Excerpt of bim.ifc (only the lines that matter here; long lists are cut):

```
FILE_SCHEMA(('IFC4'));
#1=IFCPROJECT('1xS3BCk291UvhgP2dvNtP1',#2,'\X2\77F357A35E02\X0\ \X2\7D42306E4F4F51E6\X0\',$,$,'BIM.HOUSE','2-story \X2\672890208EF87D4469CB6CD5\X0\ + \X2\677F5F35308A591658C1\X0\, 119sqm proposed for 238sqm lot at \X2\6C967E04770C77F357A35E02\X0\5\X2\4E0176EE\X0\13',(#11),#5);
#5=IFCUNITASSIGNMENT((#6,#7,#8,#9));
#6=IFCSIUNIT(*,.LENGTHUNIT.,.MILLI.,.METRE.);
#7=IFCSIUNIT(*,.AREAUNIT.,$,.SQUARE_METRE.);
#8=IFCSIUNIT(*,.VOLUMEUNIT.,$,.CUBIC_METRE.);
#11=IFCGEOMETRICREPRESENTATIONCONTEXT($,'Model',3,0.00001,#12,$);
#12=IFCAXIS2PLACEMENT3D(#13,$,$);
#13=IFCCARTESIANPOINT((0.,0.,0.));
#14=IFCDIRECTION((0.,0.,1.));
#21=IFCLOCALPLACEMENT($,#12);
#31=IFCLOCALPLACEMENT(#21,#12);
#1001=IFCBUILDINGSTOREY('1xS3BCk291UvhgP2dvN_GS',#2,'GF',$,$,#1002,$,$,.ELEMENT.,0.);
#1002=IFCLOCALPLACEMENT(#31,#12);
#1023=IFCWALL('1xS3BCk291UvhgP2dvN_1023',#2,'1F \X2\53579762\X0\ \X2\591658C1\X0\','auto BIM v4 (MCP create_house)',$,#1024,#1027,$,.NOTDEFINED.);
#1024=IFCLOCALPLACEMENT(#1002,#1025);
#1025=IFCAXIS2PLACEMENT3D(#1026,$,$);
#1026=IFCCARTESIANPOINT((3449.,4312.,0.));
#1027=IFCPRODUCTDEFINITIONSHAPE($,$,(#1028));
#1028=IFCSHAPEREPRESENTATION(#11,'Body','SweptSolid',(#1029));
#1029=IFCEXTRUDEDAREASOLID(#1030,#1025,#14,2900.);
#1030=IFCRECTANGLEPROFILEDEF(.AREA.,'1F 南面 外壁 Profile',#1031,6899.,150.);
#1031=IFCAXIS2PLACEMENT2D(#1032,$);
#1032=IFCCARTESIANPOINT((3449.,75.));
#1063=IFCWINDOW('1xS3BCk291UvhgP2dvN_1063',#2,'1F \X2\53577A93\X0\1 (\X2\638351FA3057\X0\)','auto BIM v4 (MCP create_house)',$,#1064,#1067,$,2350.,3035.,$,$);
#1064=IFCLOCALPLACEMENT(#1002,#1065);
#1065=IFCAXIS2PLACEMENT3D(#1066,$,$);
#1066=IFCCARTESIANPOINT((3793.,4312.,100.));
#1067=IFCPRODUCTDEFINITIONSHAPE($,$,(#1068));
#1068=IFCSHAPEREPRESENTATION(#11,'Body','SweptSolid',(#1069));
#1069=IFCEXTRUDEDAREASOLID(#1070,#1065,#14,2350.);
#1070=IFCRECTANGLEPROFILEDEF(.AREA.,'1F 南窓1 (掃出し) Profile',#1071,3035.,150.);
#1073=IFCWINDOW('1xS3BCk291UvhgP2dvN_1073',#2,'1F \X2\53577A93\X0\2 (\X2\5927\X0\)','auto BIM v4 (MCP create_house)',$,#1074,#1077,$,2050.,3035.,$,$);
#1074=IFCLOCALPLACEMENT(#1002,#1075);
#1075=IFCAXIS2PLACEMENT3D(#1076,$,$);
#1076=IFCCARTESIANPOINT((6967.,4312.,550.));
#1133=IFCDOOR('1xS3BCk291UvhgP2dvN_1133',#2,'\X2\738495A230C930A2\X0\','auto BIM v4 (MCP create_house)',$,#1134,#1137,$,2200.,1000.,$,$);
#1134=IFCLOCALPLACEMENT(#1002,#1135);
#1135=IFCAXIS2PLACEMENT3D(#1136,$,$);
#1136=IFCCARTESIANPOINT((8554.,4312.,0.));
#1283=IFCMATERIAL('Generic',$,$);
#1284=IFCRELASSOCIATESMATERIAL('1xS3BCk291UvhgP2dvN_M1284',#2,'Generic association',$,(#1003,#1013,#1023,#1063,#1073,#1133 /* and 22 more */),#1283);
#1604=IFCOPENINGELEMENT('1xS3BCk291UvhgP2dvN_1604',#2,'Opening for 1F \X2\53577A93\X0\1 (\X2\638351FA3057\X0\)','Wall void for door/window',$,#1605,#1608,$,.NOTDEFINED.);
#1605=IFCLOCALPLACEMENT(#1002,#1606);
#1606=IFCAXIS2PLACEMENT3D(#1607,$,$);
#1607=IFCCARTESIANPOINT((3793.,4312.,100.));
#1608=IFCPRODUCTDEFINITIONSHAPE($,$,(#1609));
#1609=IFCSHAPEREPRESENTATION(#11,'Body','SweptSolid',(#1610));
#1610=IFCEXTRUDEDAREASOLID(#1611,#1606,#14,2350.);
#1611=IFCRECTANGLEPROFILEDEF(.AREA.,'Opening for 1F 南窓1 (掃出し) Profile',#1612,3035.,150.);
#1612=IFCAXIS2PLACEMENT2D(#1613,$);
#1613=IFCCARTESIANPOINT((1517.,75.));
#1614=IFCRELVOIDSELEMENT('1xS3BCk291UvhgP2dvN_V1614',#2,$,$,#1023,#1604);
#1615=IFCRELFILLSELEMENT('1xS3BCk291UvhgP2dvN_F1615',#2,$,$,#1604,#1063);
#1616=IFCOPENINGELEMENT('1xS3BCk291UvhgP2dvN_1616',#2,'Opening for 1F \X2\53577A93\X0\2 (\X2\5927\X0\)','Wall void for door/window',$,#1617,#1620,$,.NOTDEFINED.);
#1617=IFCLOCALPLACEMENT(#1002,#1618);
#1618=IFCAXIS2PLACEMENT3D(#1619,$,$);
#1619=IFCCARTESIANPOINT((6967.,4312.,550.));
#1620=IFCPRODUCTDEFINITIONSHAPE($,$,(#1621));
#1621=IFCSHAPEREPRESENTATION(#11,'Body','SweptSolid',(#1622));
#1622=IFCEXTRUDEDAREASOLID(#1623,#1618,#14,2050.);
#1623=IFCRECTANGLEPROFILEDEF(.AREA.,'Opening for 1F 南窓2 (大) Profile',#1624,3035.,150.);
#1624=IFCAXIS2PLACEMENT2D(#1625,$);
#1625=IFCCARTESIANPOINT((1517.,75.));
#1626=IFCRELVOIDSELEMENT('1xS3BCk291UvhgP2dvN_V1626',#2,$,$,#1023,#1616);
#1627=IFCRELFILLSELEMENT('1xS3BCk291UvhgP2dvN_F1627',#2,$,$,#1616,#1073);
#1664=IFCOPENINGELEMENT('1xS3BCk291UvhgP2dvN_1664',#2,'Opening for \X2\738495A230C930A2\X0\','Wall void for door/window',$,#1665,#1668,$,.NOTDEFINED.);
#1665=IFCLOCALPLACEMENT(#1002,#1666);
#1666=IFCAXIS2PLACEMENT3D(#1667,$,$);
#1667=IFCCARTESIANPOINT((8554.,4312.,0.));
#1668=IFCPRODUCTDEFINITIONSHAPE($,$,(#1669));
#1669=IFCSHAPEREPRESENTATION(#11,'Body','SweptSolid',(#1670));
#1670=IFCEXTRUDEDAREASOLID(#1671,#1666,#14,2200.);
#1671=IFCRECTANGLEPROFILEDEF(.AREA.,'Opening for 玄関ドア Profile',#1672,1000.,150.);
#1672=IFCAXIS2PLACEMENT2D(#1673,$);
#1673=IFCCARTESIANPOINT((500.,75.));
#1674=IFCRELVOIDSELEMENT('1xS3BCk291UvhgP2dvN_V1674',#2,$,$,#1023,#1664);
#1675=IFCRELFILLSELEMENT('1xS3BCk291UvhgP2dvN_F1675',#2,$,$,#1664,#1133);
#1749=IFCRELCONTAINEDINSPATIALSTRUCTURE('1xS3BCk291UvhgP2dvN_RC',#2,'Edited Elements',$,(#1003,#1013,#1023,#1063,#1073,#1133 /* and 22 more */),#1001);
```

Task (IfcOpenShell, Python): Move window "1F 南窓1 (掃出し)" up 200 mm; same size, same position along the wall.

```python
import numpy as np
import ifcopenshell
import ifcopenshell.api.geometry
import ifcopenshell.util.placement
import ifcopenshell.util.unit

model = ifcopenshell.open("bim.ifc")
unit_scale = ifcopenshell.util.unit.calculate_unit_scale(model)

window = model.by_id(1063)
opening = window.FillsVoids[0].RelatingOpeningElement
dz = 200.0

shift = np.array([0.0, 0.0, dz])
# The window is not placed relative to its opening, so move both.
for product in (opening, window):
    matrix = ifcopenshell.util.placement.get_local_placement(product.ObjectPlacement)
    matrix[:3, 3] += shift
    ifcopenshell.api.geometry.edit_object_placement(model, product=product, matrix=matrix, is_si=False)

print(f"moved by {dz * unit_scale:+.3f} m")

model.write("bim_updated.ifc")
```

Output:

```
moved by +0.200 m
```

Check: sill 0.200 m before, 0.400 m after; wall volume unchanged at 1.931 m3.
